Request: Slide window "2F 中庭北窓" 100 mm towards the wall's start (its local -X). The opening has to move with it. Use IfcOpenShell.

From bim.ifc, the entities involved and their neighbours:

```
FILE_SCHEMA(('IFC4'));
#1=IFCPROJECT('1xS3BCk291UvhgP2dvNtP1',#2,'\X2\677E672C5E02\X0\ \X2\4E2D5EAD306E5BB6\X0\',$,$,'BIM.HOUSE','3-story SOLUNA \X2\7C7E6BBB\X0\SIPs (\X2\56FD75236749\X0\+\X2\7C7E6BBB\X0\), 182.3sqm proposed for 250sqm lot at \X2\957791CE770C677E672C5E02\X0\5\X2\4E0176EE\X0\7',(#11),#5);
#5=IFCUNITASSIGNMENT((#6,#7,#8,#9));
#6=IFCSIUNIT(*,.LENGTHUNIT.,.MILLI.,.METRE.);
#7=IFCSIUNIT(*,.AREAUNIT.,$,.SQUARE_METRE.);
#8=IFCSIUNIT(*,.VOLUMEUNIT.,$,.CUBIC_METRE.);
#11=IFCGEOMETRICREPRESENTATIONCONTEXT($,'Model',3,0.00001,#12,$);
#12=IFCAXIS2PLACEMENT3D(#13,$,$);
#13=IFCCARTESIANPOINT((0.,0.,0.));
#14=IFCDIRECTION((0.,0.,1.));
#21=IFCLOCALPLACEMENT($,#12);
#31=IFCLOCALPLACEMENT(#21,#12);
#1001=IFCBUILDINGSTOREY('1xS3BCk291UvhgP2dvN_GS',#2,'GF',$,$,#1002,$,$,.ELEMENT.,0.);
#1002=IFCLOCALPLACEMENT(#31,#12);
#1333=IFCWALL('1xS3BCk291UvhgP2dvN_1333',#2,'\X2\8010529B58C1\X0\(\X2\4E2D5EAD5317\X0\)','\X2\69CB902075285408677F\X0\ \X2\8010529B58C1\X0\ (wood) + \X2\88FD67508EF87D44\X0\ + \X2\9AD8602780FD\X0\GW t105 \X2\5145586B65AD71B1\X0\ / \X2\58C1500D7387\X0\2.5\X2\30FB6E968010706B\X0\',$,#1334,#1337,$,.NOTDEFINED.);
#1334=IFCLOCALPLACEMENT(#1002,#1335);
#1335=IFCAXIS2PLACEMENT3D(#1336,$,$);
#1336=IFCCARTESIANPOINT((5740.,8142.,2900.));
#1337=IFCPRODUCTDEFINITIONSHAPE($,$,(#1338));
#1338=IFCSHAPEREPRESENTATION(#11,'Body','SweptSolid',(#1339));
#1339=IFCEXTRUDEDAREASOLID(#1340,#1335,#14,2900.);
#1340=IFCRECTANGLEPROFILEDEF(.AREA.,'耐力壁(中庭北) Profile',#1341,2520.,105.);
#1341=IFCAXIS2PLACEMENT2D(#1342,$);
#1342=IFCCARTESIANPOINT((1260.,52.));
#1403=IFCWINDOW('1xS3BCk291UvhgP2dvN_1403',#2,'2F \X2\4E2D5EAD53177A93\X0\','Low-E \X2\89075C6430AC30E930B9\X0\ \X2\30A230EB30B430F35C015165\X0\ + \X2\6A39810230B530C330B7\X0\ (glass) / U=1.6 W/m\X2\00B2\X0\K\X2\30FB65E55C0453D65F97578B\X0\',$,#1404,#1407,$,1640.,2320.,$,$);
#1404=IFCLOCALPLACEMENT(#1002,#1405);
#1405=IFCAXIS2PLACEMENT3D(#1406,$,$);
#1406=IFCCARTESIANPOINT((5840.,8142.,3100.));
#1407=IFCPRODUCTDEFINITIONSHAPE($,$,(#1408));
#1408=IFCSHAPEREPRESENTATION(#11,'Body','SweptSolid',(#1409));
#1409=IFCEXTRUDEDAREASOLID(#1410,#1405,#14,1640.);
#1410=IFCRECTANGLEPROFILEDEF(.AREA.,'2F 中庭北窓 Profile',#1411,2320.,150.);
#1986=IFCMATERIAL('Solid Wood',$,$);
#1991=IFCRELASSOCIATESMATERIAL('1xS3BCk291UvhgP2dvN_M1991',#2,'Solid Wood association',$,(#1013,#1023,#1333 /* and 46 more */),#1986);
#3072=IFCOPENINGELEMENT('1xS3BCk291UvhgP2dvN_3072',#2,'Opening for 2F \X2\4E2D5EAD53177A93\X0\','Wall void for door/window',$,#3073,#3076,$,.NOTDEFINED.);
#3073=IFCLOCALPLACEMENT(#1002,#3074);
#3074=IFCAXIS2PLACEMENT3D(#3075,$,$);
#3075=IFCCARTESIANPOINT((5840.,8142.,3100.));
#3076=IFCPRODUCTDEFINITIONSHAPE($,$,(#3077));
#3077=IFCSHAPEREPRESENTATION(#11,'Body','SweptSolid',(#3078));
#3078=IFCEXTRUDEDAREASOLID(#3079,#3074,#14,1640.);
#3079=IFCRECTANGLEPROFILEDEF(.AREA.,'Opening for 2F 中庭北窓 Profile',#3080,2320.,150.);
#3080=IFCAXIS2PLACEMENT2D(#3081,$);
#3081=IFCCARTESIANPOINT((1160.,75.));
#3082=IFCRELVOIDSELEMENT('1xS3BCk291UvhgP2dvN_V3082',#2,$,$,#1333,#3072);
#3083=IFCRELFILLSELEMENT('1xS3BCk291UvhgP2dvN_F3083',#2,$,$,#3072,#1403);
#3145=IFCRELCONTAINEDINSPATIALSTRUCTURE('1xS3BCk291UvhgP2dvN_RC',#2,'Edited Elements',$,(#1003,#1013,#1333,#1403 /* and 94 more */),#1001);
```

```python
import ifcopenshell
import ifcopenshell.api.geometry
import ifcopenshell.util.placement

model = ifcopenshell.open("bim.ifc")

window = model.by_guid("1xS3BCk291UvhgP2dvN_1403")
opening = window.FillsVoids[0].RelatingOpeningElement
wall = opening.VoidsElements[0].RelatingBuildingElement

wall_matrix = ifcopenshell.util.placement.get_local_placement(wall.ObjectPlacement)
shift = wall_matrix[:3, 0] * -100.0
before = ifcopenshell.util.placement.get_local_placement(window.ObjectPlacement)[:3, 3].copy()

# The window is not placed relative to its opening, so move both.
for product in (opening, window):
    matrix = ifcopenshell.util.placement.get_local_placement(product.ObjectPlacement)
    matrix[:3, 3] += shift
    ifcopenshell.api.geometry.edit_object_placement(model, product=product, matrix=matrix, is_si=False)

after = ifcopenshell.util.placement.get_local_placement(window.ObjectPlacement)[:3, 3]
print("window moved by", (after - before).round(3) + 0.0)

model.write("bim_v2.ifc")
```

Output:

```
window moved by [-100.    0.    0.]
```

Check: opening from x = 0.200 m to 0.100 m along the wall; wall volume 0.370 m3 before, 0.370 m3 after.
